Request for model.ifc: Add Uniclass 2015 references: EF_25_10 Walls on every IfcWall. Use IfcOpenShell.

First a look at what the model holds.

```python
import ifcopenshell

model = ifcopenshell.open("model.ifc")
print(model.schema)
print("classifications:", [c.Name for c in model.by_type("IfcClassification")])
for ifc_class in ("IfcDoor", "IfcRoof", "IfcStair", "IfcWall", "IfcWindow"):
    print(ifc_class, len(model.by_type(ifc_class)))
```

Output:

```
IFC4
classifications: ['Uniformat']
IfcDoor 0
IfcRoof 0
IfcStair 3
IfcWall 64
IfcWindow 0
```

```python
import ifcopenshell
import ifcopenshell.api.classification

model = ifcopenshell.open("model.ifc")

system = ifcopenshell.api.classification.add_classification(model, classification="Uniclass 2015")

codes = {
    "IfcWall": ("EF_25_10", "Walls"),
}
for ifc_class, (code, name) in codes.items():
    products = model.by_type(ifc_class)
    ifcopenshell.api.classification.add_reference(
        model, products=products, classification=system, identification=code, name=name
    )
    print(code, len(products))

model.write("model_edited.ifc")
```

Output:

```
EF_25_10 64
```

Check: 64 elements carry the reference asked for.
